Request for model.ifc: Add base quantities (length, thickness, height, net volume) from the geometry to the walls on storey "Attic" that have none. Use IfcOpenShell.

First a look at what the model holds.

```python
import ifcopenshell
import ifcopenshell.util.element
import ifcopenshell.util.unit

model = ifcopenshell.open("model.ifc")
print(model.schema)
for unit_type in ("LENGTHUNIT", "AREAUNIT", "VOLUMEUNIT"):
    print(unit_type, ifcopenshell.util.unit.calculate_unit_scale(model, unit_type))
storey = next(s for s in model.by_type("IfcBuildingStorey") if s.Name == "Attic")
walls = [e for e in ifcopenshell.util.element.get_decomposition(storey) if e.is_a("IfcWall")]
for e in sorted(walls, key=lambda e: e.id()):
    print(e.id(), e.is_a(), e.Name, list(ifcopenshell.util.element.get_psets(e, qtos_only=True)), sep=" | ")
```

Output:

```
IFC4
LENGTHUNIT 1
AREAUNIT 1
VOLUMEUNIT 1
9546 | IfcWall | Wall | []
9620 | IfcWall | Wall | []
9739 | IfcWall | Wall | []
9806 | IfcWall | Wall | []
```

```python
import ifcopenshell
import ifcopenshell.api.pset
import ifcopenshell.geom
import ifcopenshell.util.element
import ifcopenshell.util.shape
import ifcopenshell.util.unit

model = ifcopenshell.open("model.ifc")
unit_scale = ifcopenshell.util.unit.calculate_unit_scale(model)
volume_scale = ifcopenshell.util.unit.calculate_unit_scale(model, "VOLUMEUNIT")
settings = ifcopenshell.geom.settings()

storey = next(s for s in model.by_type("IfcBuildingStorey") if s.Name == "Attic")
walls = [e for e in ifcopenshell.util.element.get_decomposition(storey) if e.is_a("IfcWall")]

for e in sorted(walls, key=lambda e: e.id()):
    if ifcopenshell.util.element.get_psets(e, qtos_only=True, should_inherit=False):
        continue
    # Geometry comes back in metres, in the element's own axes.
    shape = ifcopenshell.geom.create_shape(settings, e)
    values = {
        "Length": ifcopenshell.util.shape.get_x(shape.geometry) / unit_scale,
        "Width": ifcopenshell.util.shape.get_y(shape.geometry) / unit_scale,
        "Height": ifcopenshell.util.shape.get_z(shape.geometry) / unit_scale,
        "NetVolume": ifcopenshell.util.shape.get_volume(shape.geometry) / volume_scale,
    }
    qto = ifcopenshell.api.pset.add_qto(model, product=e, name="Qto_WallBaseQuantities")
    ifcopenshell.api.pset.edit_qto(model, qto=qto, properties=values)
    print(e.id(), {k: round(v, 3) for k, v in values.items()})

model.write("model_updated.ifc")
```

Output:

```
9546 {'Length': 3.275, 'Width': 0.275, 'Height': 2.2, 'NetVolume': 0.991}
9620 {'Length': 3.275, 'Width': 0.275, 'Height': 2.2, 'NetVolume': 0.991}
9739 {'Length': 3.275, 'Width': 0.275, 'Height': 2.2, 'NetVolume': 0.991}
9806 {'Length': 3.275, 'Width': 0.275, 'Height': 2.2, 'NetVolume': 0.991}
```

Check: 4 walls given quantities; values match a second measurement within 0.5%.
